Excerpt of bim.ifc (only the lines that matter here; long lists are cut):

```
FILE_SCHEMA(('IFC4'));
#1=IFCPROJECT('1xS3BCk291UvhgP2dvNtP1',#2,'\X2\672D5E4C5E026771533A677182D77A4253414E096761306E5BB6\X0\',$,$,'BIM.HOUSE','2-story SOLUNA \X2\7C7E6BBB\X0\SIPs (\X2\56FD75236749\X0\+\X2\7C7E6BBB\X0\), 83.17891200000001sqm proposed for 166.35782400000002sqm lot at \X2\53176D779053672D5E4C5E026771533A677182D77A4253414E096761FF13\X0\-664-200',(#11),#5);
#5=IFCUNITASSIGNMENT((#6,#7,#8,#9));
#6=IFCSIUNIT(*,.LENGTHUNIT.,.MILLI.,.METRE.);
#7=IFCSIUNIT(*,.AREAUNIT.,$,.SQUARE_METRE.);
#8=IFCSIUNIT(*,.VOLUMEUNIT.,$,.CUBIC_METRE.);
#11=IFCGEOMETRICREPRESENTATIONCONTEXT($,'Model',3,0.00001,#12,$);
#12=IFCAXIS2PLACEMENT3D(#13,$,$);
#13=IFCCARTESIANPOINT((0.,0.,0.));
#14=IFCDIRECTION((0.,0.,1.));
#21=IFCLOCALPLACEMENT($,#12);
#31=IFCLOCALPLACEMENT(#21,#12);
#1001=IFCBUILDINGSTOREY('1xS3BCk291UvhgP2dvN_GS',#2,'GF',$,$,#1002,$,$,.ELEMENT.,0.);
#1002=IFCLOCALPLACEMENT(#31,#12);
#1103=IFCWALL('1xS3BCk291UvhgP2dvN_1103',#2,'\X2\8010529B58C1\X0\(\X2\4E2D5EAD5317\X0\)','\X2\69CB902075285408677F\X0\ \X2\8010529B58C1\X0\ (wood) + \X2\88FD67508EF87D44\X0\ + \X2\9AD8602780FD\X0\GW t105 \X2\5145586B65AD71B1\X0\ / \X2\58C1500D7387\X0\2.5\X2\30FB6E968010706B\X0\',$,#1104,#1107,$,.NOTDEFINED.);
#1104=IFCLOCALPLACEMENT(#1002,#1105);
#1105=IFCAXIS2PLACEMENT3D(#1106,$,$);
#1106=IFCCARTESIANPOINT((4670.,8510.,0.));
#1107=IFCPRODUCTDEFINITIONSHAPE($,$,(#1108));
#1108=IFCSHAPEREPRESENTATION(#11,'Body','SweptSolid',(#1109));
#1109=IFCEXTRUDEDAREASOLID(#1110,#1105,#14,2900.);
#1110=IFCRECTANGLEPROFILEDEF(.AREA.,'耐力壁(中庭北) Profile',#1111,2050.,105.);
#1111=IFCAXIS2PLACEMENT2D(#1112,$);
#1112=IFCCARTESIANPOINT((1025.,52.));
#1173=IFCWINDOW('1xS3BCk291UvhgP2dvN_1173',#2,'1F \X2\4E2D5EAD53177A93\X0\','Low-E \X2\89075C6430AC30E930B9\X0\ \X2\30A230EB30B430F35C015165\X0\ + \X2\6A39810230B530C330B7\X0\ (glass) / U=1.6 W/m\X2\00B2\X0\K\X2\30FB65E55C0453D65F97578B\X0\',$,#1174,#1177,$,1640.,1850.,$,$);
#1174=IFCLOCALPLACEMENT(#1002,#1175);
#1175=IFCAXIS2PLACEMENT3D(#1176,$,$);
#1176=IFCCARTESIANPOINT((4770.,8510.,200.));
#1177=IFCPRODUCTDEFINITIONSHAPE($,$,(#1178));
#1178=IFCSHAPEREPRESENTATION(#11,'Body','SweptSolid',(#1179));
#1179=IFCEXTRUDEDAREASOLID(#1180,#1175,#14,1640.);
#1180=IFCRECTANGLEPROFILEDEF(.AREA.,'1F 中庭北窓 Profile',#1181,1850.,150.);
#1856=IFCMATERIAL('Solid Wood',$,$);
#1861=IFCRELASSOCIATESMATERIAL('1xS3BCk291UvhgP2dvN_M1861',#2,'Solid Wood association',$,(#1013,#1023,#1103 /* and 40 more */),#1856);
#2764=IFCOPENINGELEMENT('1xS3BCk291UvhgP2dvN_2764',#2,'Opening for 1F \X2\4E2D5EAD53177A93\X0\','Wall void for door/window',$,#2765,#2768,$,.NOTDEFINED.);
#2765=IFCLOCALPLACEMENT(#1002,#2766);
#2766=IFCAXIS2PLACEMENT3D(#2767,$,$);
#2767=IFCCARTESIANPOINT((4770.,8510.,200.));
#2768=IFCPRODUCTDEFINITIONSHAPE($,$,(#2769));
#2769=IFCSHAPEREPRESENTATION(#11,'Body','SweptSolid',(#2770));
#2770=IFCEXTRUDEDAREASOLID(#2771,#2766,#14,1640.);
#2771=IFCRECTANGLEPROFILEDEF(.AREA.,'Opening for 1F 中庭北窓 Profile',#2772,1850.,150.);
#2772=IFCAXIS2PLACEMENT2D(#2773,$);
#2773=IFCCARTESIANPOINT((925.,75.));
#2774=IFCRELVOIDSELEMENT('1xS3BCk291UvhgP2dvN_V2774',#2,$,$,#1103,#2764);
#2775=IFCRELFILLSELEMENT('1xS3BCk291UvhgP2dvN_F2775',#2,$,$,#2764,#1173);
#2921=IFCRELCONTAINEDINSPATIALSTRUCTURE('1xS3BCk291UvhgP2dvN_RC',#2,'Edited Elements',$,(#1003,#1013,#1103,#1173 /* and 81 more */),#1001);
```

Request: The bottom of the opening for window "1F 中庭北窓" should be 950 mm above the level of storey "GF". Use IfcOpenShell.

```python
import numpy as np
import ifcopenshell
import ifcopenshell.api.geometry
import ifcopenshell.geom
import ifcopenshell.util.element
import ifcopenshell.util.placement
import ifcopenshell.util.shape
import ifcopenshell.util.unit

model = ifcopenshell.open("bim.ifc")
unit_scale = ifcopenshell.util.unit.calculate_unit_scale(model)

window = model.by_id(1173)
opening = window.FillsVoids[0].RelatingOpeningElement
storey = ifcopenshell.util.element.get_container(window, ifc_class="IfcBuildingStorey")
level = ifcopenshell.util.placement.get_local_placement(storey.ObjectPlacement)[2, 3]

# The opening's origin need not be at the sill, so measure its lowest point.
shape = ifcopenshell.geom.create_shape(ifcopenshell.geom.settings(), opening)
bottom = ifcopenshell.util.shape.get_shape_bottom_elevation(shape, shape.geometry) / unit_scale
dz = level + 0.95 / unit_scale - bottom

shift = np.array([0.0, 0.0, dz])
# The window is not placed relative to its opening, so move both.
for product in (opening, window):
    matrix = ifcopenshell.util.placement.get_local_placement(product.ObjectPlacement)
    matrix[:3, 3] += shift
    ifcopenshell.api.geometry.edit_object_placement(model, product=product, matrix=matrix, is_si=False)

print(f"moved by {dz * unit_scale:+.3f} m")

model.write("bim_rev.ifc")
```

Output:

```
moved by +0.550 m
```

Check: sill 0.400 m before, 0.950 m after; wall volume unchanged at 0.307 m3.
